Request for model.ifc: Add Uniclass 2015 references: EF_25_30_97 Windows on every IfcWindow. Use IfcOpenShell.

First a look at what the model holds.

```python
import ifcopenshell

model = ifcopenshell.open("model.ifc")
print(model.schema)
print("classifications:", [c.Name for c in model.by_type("IfcClassification")])
for ifc_class in ("IfcDoor", "IfcRoof", "IfcStair", "IfcWall", "IfcWindow"):
    print(ifc_class, len(model.by_type(ifc_class)))
```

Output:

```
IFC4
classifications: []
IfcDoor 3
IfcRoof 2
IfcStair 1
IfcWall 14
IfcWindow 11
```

```python
import ifcopenshell
import ifcopenshell.api.classification

model = ifcopenshell.open("model.ifc")

system = ifcopenshell.api.classification.add_classification(model, classification="Uniclass 2015")

codes = {
    "IfcWindow": ("EF_25_30_97", "Windows"),
}
for ifc_class, (code, name) in codes.items():
    products = model.by_type(ifc_class)
    ifcopenshell.api.classification.add_reference(
        model, products=products, classification=system, identification=code, name=name
    )
    print(code, len(products))

model.write("model-out.ifc")
```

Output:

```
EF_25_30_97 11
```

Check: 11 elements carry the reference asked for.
